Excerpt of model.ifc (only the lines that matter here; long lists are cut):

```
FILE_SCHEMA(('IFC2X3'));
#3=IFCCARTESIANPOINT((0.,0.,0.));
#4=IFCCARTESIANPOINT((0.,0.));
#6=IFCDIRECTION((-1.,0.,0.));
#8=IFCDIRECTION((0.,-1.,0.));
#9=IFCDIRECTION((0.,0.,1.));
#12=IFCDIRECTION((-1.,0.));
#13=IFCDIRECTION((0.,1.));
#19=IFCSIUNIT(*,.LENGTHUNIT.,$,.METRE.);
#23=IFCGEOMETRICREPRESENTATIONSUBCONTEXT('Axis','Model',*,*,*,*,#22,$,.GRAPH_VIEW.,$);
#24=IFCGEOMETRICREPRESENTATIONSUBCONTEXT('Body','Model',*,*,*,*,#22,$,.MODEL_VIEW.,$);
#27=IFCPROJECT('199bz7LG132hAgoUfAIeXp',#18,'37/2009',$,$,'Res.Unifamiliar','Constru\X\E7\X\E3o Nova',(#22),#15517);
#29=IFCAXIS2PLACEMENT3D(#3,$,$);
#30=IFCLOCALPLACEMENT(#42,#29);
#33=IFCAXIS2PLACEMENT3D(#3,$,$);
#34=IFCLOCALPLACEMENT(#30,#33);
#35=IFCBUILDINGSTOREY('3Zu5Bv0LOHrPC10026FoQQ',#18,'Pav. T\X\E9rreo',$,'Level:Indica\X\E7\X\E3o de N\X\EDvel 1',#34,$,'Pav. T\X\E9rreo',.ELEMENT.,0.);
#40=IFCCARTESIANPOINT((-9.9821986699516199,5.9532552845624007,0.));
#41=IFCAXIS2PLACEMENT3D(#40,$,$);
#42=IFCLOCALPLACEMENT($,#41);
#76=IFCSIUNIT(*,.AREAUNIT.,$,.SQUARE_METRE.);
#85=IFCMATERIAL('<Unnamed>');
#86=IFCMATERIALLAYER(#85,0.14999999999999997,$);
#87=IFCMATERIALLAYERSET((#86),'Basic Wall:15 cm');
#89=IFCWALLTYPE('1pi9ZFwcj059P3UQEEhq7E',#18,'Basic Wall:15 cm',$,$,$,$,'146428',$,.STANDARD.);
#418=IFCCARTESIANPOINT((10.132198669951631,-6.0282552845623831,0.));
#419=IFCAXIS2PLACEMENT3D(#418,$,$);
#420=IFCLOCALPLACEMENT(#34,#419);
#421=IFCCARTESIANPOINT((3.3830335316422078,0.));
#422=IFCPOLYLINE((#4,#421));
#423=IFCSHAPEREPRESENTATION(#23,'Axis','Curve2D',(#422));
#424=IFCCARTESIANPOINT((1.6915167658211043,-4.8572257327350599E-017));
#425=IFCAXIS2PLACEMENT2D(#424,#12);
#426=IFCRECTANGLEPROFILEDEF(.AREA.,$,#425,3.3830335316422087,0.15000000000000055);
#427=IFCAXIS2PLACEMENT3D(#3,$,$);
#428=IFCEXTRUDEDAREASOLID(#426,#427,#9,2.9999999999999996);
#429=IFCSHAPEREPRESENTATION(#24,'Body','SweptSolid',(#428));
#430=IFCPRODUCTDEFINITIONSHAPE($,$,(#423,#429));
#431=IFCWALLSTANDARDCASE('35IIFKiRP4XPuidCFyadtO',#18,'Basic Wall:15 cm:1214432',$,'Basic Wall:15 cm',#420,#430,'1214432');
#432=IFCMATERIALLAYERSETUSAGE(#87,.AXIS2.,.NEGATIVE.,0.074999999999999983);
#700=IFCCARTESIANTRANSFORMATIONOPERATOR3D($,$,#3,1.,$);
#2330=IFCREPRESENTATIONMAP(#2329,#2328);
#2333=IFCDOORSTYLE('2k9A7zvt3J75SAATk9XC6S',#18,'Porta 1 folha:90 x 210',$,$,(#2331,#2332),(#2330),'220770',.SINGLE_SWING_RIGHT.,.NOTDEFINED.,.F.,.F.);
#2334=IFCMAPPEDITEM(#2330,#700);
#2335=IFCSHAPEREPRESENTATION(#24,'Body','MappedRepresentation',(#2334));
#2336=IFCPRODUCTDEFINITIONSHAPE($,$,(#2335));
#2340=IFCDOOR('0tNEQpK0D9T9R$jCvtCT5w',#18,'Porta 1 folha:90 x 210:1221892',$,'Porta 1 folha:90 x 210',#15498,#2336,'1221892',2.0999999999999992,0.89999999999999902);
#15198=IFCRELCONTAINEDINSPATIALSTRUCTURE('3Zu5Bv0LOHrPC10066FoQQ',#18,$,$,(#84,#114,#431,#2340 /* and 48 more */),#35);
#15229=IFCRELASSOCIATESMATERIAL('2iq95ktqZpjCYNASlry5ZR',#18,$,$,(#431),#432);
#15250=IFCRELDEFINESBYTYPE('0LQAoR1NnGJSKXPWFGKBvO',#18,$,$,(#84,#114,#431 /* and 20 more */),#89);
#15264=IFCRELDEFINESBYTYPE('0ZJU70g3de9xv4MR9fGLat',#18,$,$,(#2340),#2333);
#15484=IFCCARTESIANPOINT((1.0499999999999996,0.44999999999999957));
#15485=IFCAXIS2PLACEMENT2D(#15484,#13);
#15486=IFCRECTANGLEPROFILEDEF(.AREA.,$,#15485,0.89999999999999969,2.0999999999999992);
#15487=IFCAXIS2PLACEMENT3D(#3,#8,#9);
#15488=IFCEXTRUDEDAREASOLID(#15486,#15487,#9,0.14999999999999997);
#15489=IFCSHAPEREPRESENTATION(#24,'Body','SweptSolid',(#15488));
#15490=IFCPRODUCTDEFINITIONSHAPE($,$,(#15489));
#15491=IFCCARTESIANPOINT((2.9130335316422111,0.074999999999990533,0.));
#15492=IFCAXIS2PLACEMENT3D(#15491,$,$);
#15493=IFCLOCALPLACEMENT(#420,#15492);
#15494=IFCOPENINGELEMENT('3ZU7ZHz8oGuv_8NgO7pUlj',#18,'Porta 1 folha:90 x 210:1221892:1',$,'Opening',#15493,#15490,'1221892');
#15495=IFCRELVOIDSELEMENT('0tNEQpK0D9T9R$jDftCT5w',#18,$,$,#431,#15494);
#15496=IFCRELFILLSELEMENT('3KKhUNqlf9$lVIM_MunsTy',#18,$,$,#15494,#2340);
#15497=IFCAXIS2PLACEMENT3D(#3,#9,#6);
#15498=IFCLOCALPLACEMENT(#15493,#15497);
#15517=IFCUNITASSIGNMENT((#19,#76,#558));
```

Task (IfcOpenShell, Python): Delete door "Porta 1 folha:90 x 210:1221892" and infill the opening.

```python
import ifcopenshell
import ifcopenshell.api.feature
import ifcopenshell.api.root
import ifcopenshell.geom
import ifcopenshell.util.shape

model = ifcopenshell.open("model.ifc")
settings = ifcopenshell.geom.settings()


def volume(element):
    """Net volume in cubic metres, openings subtracted."""
    shape = ifcopenshell.geom.create_shape(settings, element)
    return ifcopenshell.util.shape.get_volume(shape.geometry)


door = model.by_guid("0tNEQpK0D9T9R$jCvtCT5w")
opening = door.FillsVoids[0].RelatingOpeningElement
wall = opening.VoidsElements[0].RelatingBuildingElement
before = volume(wall)

ifcopenshell.api.root.remove_product(model, product=door)
ifcopenshell.api.feature.remove_feature(model, feature=opening)

after = volume(wall)

print(f"wall volume {before:.3f} -> {after:.3f} m3")

model.write("model_updated.ifc")
```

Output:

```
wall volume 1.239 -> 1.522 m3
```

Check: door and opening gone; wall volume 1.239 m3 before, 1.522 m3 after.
